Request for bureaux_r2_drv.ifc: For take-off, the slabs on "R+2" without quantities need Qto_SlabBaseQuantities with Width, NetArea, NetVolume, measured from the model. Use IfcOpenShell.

First a look at what the model holds.

```python
import ifcopenshell
import ifcopenshell.util.element
import ifcopenshell.util.unit

model = ifcopenshell.open("bureaux_r2_drv.ifc")
print(model.schema)
for unit_type in ("LENGTHUNIT", "AREAUNIT", "VOLUMEUNIT"):
    print(unit_type, ifcopenshell.util.unit.calculate_unit_scale(model, unit_type))
storey = next(s for s in model.by_type("IfcBuildingStorey") if s.Name == "R+2")
slabs = [e for e in ifcopenshell.util.element.get_decomposition(storey) if e.is_a("IfcSlab")]
for e in sorted(slabs, key=lambda e: e.id()):
    print(e.id(), e.is_a(), e.Name, list(ifcopenshell.util.element.get_psets(e, qtos_only=True)), sep=" | ")
```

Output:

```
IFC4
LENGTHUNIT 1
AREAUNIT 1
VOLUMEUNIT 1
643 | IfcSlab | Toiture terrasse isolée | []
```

```python
import ifcopenshell
import ifcopenshell.api.pset
import ifcopenshell.geom
import ifcopenshell.util.element
import ifcopenshell.util.shape
import ifcopenshell.util.unit

model = ifcopenshell.open("bureaux_r2_drv.ifc")
unit_scale = ifcopenshell.util.unit.calculate_unit_scale(model)
area_scale = ifcopenshell.util.unit.calculate_unit_scale(model, "AREAUNIT")
volume_scale = ifcopenshell.util.unit.calculate_unit_scale(model, "VOLUMEUNIT")
settings = ifcopenshell.geom.settings()

storey = next(s for s in model.by_type("IfcBuildingStorey") if s.Name == "R+2")
slabs = [e for e in ifcopenshell.util.element.get_decomposition(storey) if e.is_a("IfcSlab")]

for e in sorted(slabs, key=lambda e: e.id()):
    if ifcopenshell.util.element.get_psets(e, qtos_only=True, should_inherit=False):
        continue
    # Geometry comes back in metres, in the element's own axes.
    shape = ifcopenshell.geom.create_shape(settings, e)
    values = {
        "Width": ifcopenshell.util.shape.get_z(shape.geometry) / unit_scale,
        "NetArea": ifcopenshell.util.shape.get_footprint_area(shape.geometry) / area_scale,
        "NetVolume": ifcopenshell.util.shape.get_volume(shape.geometry) / volume_scale,
    }
    qto = ifcopenshell.api.pset.add_qto(model, product=e, name="Qto_SlabBaseQuantities")
    ifcopenshell.api.pset.edit_qto(model, qto=qto, properties=values)
    print(e.id(), {k: round(v, 3) for k, v in values.items()})

model.write("bureaux_r2_drv_edited.ifc")
```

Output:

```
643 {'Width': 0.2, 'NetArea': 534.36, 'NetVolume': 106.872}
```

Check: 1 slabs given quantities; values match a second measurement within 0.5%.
